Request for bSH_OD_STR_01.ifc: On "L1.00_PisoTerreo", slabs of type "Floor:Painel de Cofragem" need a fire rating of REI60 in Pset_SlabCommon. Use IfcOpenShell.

First a look at what the model holds.

```python
import ifcopenshell
import ifcopenshell.util.element

model = ifcopenshell.open("bSH_OD_STR_01.ifc")
print(model.schema)
storey = next(s for s in model.by_type("IfcBuildingStorey") if s.Name == "L1.00_PisoTerreo")
slabs = [e for e in ifcopenshell.util.element.get_decomposition(storey) if e.is_a("IfcSlab")]
seen = {}
for e in slabs:
    element_type = ifcopenshell.util.element.get_type(e)
    key = (element_type.Name if element_type != e and element_type else None, ifcopenshell.util.element.get_pset(e, "Pset_SlabCommon", "FireRating"))
    seen[key] = seen.get(key, 0) + 1
for (name, value), count in sorted(seen.items(), key=str):
    print(count, "x", name, "|", value)
```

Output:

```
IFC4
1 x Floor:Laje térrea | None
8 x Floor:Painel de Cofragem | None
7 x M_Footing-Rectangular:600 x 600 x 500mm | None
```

```python
import ifcopenshell
import ifcopenshell.api.pset
import ifcopenshell.util.element

model = ifcopenshell.open("bSH_OD_STR_01.ifc")

storey = next(s for s in model.by_type("IfcBuildingStorey") if s.Name == "L1.00_PisoTerreo")
slabs = [e for e in ifcopenshell.util.element.get_decomposition(storey) if e.is_a("IfcSlab")]

count = 0
for e in slabs:
    element_type = ifcopenshell.util.element.get_type(e)
    if element_type in (None, e) or element_type.Name != "Floor:Painel de Cofragem":
        continue
    # add_pset returns the element's existing set when there is one.
    pset = ifcopenshell.api.pset.add_pset(model, product=e, name="Pset_SlabCommon")
    ifcopenshell.api.pset.edit_pset(model, pset=pset, properties={"FireRating": "REI60"})
    count += 1

print(count, "slabs updated")

model.write("bSH_OD_STR_01_updated.ifc")
```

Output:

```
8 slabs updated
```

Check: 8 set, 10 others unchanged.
